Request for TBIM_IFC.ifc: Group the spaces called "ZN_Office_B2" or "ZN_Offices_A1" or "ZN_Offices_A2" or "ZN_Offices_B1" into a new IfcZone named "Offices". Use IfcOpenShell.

First a look at what the model holds.

```python
import ifcopenshell

model = ifcopenshell.open("TBIM_IFC.ifc")
print(model.schema)
seen = {}
for space in model.by_type("IfcSpace"):
    seen[space.LongName] = seen.get(space.LongName, 0) + 1
for name, count in sorted(seen.items(), key=str):
    print(count, "x", name)
print("zones:", [z.Name for z in model.by_type("IfcZone")][:20])
```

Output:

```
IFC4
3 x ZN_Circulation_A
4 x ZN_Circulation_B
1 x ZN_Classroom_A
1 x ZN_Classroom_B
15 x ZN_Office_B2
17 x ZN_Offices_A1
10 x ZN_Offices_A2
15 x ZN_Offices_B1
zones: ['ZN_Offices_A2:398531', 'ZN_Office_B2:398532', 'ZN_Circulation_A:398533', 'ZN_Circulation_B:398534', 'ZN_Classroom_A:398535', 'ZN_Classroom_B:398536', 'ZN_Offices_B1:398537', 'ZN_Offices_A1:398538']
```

```python
import ifcopenshell
import ifcopenshell.api.group
import ifcopenshell.api.root

model = ifcopenshell.open("TBIM_IFC.ifc")

names = {"ZN_Office_B2", "ZN_Offices_A1", "ZN_Offices_A2", "ZN_Offices_B1"}
spaces = [s for s in model.by_type("IfcSpace") if s.LongName in names]

zone = ifcopenshell.api.root.create_entity(model, ifc_class="IfcZone", name="Offices")
ifcopenshell.api.group.assign_group(model, products=spaces, group=zone)
print(len(spaces), "spaces in", zone.Name)

model.write("TBIM_IFC_rev.ifc")
```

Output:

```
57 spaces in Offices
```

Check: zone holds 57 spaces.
